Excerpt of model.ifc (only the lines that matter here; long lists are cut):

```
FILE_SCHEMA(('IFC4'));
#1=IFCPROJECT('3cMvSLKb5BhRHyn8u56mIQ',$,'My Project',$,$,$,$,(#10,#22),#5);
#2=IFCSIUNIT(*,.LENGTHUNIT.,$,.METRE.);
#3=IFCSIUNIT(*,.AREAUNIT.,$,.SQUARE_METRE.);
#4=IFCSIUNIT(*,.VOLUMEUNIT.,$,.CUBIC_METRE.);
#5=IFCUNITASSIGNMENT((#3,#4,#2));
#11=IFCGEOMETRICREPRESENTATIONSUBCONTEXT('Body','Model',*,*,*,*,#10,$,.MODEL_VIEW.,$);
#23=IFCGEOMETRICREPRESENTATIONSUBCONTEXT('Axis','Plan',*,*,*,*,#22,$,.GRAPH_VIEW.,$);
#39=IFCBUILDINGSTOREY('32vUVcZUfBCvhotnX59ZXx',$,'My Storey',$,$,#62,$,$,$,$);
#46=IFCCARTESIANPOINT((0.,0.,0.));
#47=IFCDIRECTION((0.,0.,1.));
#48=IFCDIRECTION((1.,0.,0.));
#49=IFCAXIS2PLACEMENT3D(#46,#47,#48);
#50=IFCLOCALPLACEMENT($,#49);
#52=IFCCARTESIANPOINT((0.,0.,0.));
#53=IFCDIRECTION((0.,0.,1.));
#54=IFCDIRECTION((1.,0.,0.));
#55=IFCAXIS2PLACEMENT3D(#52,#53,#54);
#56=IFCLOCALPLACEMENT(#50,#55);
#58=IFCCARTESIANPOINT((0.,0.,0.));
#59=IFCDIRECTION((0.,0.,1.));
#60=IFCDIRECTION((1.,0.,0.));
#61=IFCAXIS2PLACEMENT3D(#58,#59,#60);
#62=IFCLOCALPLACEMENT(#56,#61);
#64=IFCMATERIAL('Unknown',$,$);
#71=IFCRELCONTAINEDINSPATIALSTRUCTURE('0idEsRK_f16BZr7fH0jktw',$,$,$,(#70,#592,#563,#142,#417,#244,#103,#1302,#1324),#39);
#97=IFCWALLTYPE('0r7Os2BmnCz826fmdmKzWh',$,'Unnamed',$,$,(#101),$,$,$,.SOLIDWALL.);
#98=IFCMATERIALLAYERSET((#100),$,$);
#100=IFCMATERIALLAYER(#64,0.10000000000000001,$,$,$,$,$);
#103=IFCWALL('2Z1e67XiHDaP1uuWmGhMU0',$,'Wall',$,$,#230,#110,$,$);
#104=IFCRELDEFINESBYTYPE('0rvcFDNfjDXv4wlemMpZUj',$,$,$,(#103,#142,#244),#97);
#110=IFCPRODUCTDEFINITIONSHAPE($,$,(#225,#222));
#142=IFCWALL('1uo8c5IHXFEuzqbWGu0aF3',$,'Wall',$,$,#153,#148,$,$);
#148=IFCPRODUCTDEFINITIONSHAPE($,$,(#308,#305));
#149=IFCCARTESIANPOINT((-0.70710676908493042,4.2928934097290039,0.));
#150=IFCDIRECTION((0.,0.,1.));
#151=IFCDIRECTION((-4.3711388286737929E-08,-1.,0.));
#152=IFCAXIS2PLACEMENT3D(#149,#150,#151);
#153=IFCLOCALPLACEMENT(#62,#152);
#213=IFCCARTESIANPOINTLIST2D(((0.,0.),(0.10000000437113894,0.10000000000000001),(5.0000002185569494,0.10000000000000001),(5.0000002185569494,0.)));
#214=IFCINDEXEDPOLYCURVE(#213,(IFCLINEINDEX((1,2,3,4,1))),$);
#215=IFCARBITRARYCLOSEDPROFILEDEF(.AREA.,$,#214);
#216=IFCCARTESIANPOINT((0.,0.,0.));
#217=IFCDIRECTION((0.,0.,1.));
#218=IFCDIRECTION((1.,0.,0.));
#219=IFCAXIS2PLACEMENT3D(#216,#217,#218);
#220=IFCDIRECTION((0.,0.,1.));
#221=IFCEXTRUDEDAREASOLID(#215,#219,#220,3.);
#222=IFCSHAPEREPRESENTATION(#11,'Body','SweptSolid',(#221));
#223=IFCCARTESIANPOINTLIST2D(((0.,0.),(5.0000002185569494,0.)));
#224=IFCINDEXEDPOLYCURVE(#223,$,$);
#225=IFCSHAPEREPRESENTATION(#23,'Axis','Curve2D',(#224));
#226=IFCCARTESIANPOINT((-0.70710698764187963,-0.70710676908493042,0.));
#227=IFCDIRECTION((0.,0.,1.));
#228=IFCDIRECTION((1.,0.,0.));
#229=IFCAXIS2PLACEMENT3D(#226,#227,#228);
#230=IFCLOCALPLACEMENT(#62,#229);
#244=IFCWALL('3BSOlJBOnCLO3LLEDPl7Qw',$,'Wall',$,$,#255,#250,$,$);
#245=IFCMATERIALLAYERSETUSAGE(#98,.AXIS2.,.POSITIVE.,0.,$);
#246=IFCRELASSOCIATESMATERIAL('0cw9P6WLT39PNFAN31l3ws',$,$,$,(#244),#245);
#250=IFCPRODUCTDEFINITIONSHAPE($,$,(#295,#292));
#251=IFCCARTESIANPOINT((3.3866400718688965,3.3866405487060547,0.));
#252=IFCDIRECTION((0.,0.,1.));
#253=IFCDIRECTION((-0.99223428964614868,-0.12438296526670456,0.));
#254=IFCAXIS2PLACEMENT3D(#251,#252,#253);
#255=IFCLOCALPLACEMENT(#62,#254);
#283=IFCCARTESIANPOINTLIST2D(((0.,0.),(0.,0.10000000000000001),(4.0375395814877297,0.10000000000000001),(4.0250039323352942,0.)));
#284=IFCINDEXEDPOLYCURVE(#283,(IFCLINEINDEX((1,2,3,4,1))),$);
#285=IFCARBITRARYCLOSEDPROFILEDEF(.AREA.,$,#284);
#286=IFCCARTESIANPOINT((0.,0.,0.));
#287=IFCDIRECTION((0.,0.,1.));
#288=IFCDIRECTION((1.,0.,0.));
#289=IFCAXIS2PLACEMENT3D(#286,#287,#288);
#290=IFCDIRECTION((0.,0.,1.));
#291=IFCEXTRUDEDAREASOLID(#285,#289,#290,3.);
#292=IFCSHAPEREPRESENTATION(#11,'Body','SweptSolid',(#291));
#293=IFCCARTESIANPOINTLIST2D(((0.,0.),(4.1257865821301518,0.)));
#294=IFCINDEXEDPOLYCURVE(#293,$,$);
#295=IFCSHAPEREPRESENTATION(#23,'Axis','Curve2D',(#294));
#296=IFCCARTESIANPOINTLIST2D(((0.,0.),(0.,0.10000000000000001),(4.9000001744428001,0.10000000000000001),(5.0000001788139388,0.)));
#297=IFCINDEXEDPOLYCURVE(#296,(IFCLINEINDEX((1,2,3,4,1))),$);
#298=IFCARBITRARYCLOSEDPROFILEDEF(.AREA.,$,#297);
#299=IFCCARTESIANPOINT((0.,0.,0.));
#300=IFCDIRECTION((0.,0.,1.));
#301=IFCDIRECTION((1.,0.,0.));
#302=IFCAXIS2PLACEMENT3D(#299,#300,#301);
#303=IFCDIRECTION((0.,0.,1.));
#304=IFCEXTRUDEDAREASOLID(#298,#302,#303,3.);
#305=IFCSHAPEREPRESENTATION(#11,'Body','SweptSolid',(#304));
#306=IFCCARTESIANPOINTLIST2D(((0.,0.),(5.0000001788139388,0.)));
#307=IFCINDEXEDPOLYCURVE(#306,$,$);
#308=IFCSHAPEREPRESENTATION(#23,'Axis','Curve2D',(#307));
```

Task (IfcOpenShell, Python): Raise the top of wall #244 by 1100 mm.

```python
import ifcopenshell
import ifcopenshell.geom
import ifcopenshell.util.representation
import ifcopenshell.util.shape
import ifcopenshell.util.unit

model = ifcopenshell.open("model.ifc")
unit_scale = ifcopenshell.util.unit.calculate_unit_scale(model)
settings = ifcopenshell.geom.settings()


def volume(element):
    """Net volume in cubic metres, openings subtracted."""
    shape = ifcopenshell.geom.create_shape(settings, element)
    return ifcopenshell.util.shape.get_volume(shape.geometry)


wall = model.by_id(244)
before = volume(wall)

body = ifcopenshell.util.representation.get_representation(wall, "Model", "Body")
solid = body.Items[0]
old_height = solid.Depth
solid.Depth += 1.1 / unit_scale
after = volume(wall)

print(f"height {old_height:g} -> {solid.Depth:g}, volume {before:.3f} -> {after:.3f} m3")

model.write("model_edited.ifc")
```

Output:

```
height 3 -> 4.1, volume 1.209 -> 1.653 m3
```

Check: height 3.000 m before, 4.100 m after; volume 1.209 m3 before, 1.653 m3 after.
